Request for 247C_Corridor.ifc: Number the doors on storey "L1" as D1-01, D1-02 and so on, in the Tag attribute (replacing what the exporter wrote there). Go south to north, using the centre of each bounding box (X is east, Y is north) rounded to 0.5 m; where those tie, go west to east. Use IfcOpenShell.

First a look at what the model holds.

```python
import ifcopenshell
import ifcopenshell.util.element
import ifcopenshell.util.placement

model = ifcopenshell.open("247C_Corridor.ifc")
print(model.schema)
storey = next(s for s in model.by_type("IfcBuildingStorey") if s.Name == "L1")
doors = [e for e in ifcopenshell.util.element.get_decomposition(storey) if e.is_a("IfcDoor")]
for e in sorted(doors, key=lambda e: e.id()):
    origin = ifcopenshell.util.placement.get_local_placement(e.ObjectPlacement)[:3, 3]
    print(e.id(), e.Tag, e.Name, origin.round(2) + 0.0, sep=" | ")
```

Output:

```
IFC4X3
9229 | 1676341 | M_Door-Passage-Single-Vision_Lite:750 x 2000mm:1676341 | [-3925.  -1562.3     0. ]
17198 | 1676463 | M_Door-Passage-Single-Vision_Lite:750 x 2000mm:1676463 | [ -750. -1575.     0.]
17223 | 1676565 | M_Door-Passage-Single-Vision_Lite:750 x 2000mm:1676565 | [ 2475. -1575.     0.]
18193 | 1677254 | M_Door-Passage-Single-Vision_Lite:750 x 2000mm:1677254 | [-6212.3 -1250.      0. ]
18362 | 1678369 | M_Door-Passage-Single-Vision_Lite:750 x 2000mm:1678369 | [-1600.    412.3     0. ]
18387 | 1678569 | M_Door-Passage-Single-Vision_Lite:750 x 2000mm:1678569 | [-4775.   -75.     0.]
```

```python
import ifcopenshell
import ifcopenshell.geom
import ifcopenshell.util.element
import ifcopenshell.util.shape

model = ifcopenshell.open("247C_Corridor.ifc")
settings = ifcopenshell.geom.settings()
settings.set("use-world-coords", True)


def centre(element):
    shape = ifcopenshell.geom.create_shape(settings, element)
    return ifcopenshell.util.shape.get_bbox_centroid(shape.geometry)


storey = next(s for s in model.by_type("IfcBuildingStorey") if s.Name == "L1")
doors = [e for e in ifcopenshell.util.element.get_decomposition(storey) if e.is_a("IfcDoor")]

# Insertion points can sit at a corner or the storey origin, so sort by the geometry (in metres).
centres = {e: centre(e) for e in doors}
doors.sort(key=lambda e: (round(centres[e][1] / 0.5), centres[e][0]))

for i, e in enumerate(doors, start=1):
    number = f"D1-{i:02d}"
    e.Tag = number
    print(e.id(), number)

model.write("247C_Corridor_edited.ifc")
```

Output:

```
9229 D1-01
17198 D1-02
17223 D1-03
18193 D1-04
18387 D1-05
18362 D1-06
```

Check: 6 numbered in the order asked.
